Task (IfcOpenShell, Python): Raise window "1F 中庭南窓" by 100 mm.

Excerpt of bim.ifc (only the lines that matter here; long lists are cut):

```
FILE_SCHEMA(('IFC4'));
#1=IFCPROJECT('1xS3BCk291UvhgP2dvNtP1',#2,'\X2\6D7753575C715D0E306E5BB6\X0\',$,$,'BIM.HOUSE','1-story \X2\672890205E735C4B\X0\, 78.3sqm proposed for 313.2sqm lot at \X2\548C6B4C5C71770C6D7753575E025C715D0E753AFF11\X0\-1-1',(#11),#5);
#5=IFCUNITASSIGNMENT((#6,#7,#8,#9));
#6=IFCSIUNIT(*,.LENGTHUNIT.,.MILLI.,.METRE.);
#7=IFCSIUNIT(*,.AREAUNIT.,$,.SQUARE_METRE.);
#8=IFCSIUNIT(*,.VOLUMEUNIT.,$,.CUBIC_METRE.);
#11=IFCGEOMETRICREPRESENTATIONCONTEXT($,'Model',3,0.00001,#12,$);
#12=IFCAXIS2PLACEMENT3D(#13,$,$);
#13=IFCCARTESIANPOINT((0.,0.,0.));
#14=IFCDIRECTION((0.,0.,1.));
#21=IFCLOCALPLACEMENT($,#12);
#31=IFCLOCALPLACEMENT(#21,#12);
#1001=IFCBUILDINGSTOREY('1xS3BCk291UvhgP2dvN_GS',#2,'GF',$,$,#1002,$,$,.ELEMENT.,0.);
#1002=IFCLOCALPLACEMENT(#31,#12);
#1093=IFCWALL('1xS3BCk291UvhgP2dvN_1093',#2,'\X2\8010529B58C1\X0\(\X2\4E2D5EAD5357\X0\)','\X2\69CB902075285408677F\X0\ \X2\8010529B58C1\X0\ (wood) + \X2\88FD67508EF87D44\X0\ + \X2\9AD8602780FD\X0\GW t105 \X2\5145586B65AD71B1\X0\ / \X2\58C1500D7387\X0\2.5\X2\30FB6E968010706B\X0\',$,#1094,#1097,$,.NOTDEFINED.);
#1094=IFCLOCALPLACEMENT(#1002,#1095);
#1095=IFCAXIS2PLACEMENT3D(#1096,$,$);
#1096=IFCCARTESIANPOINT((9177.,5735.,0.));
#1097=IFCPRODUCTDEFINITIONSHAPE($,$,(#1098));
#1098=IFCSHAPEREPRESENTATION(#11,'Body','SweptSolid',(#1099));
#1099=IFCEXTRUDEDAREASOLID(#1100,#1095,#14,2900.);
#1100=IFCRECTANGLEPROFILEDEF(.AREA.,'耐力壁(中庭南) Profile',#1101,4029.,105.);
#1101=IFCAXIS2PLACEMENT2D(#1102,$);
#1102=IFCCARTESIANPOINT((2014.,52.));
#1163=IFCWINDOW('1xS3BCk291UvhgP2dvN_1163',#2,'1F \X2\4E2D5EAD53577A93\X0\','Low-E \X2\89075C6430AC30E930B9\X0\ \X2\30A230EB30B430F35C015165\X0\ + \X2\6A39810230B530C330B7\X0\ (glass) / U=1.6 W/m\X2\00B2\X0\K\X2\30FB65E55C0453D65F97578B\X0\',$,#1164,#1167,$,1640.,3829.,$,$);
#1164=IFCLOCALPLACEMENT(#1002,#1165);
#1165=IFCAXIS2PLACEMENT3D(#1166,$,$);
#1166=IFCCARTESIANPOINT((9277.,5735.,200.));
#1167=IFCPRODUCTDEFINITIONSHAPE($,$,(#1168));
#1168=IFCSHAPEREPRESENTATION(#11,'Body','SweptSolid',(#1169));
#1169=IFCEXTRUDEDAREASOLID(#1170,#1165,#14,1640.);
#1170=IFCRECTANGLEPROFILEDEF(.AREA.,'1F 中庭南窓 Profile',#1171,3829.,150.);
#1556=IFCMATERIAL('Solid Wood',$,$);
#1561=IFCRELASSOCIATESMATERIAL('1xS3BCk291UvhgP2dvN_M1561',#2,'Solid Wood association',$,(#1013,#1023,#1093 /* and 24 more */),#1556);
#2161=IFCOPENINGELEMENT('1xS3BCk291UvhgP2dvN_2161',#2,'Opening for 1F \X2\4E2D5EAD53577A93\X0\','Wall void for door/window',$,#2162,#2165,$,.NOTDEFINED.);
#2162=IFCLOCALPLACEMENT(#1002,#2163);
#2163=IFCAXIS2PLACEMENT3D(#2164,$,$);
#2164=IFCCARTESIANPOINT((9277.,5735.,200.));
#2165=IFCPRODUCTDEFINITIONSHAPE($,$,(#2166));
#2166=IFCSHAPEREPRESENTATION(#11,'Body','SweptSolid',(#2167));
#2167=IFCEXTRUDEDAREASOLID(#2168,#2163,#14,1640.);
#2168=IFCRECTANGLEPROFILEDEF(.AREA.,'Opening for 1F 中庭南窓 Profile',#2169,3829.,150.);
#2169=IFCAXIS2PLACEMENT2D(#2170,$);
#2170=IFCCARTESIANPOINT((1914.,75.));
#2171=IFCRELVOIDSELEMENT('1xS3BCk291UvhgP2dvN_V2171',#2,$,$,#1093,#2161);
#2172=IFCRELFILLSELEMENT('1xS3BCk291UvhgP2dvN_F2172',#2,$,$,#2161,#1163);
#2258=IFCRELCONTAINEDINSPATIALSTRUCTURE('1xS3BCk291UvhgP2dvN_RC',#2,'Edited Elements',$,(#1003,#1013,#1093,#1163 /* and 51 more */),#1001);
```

```python
import numpy as np
import ifcopenshell
import ifcopenshell.api.geometry
import ifcopenshell.util.placement
import ifcopenshell.util.unit

model = ifcopenshell.open("bim.ifc")
unit_scale = ifcopenshell.util.unit.calculate_unit_scale(model)

window = model.by_id(1163)
opening = window.FillsVoids[0].RelatingOpeningElement
dz = 100.0

shift = np.array([0.0, 0.0, dz])
# The window is not placed relative to its opening, so move both.
for product in (opening, window):
    matrix = ifcopenshell.util.placement.get_local_placement(product.ObjectPlacement)
    matrix[:3, 3] += shift
    ifcopenshell.api.geometry.edit_object_placement(model, product=product, matrix=matrix, is_si=False)

print(f"moved by {dz * unit_scale:+.3f} m")

model.write("bim_rev.ifc")
```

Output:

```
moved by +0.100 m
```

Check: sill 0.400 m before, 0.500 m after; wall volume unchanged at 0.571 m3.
